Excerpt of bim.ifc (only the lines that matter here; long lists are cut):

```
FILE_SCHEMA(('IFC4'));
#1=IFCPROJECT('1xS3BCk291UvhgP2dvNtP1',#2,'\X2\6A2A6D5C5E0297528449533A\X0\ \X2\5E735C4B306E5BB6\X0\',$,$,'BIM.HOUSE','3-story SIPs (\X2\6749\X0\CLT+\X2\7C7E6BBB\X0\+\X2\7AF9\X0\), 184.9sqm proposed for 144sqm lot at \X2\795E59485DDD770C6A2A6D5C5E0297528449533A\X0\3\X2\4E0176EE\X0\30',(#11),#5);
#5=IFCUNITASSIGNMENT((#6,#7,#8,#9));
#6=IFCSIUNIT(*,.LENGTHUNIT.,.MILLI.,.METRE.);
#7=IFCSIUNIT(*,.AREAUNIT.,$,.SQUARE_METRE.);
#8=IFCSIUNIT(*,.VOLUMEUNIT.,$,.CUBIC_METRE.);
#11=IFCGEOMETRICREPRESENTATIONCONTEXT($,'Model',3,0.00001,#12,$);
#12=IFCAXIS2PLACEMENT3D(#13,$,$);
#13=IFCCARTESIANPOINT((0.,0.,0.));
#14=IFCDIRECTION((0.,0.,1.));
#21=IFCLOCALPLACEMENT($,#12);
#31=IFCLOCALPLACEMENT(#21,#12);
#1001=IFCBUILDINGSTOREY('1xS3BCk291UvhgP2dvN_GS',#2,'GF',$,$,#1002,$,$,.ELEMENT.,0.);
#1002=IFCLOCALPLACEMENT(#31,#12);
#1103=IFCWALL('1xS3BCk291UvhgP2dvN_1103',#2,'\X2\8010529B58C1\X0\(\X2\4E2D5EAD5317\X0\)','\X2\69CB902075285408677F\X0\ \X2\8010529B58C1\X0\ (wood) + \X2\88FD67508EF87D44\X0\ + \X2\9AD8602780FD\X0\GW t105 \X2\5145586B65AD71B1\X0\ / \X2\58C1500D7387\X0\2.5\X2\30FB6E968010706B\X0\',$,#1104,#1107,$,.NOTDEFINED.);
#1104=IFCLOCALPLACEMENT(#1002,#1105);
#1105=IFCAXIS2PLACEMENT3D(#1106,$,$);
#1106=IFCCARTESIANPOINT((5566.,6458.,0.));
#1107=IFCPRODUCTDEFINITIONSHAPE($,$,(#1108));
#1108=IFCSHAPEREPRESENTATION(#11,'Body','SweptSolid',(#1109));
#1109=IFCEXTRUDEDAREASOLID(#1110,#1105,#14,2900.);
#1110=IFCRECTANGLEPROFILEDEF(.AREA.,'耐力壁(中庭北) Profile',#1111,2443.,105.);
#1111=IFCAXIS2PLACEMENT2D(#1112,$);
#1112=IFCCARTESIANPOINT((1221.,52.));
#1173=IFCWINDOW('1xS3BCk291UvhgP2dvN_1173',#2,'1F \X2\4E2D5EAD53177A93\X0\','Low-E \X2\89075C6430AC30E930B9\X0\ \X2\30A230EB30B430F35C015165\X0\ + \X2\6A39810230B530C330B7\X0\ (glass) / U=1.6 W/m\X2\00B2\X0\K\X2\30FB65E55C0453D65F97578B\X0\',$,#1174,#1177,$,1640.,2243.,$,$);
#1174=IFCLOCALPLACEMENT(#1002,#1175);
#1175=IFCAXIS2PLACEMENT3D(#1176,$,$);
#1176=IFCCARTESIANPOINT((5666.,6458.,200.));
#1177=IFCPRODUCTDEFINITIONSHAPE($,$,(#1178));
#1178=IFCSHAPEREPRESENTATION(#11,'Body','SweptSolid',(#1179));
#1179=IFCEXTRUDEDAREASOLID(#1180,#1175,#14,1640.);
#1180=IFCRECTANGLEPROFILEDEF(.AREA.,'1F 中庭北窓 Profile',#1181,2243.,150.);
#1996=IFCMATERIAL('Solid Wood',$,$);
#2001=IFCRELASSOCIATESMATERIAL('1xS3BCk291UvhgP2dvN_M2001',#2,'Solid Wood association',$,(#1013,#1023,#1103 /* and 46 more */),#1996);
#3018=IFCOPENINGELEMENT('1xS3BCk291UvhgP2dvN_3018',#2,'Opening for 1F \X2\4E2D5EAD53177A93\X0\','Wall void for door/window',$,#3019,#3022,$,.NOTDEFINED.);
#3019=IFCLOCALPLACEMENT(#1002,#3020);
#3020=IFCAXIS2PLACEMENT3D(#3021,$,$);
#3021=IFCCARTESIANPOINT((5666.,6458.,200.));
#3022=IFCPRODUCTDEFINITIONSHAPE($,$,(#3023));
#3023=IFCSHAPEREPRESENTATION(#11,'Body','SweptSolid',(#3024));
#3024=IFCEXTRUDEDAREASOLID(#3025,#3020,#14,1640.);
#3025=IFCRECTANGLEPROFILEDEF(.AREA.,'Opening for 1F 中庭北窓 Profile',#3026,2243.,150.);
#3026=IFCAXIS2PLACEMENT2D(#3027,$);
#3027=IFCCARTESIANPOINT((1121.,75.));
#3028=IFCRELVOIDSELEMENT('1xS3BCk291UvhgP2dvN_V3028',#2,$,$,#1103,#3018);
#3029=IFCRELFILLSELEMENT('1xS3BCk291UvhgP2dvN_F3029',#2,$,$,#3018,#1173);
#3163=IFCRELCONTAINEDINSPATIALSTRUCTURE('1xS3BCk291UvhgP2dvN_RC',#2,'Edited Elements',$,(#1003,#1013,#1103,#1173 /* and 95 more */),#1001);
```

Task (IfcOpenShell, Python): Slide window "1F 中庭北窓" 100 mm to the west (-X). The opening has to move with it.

```python
import ifcopenshell
import ifcopenshell.api.geometry
import ifcopenshell.util.placement
import ifcopenshell.util.unit

model = ifcopenshell.open("bim.ifc")
unit_scale = ifcopenshell.util.unit.calculate_unit_scale(model)

window = model.by_guid("1xS3BCk291UvhgP2dvN_1173")
opening = window.FillsVoids[0].RelatingOpeningElement
wall = opening.VoidsElements[0].RelatingBuildingElement

wall_matrix = ifcopenshell.util.placement.get_local_placement(wall.ObjectPlacement)
shift = wall_matrix[:3, 0] * -0.1 / unit_scale
before = ifcopenshell.util.placement.get_local_placement(window.ObjectPlacement)[:3, 3].copy()

# The window is not placed relative to its opening, so move both.
for product in (opening, window):
    matrix = ifcopenshell.util.placement.get_local_placement(product.ObjectPlacement)
    matrix[:3, 3] += shift
    ifcopenshell.api.geometry.edit_object_placement(model, product=product, matrix=matrix, is_si=False)

after = ifcopenshell.util.placement.get_local_placement(window.ObjectPlacement)[:3, 3]
print("window moved by", (after - before).round(3) + 0.0)

model.write("bim_updated.ifc")
```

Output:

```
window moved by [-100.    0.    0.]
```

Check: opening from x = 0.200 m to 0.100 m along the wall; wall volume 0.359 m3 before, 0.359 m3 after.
